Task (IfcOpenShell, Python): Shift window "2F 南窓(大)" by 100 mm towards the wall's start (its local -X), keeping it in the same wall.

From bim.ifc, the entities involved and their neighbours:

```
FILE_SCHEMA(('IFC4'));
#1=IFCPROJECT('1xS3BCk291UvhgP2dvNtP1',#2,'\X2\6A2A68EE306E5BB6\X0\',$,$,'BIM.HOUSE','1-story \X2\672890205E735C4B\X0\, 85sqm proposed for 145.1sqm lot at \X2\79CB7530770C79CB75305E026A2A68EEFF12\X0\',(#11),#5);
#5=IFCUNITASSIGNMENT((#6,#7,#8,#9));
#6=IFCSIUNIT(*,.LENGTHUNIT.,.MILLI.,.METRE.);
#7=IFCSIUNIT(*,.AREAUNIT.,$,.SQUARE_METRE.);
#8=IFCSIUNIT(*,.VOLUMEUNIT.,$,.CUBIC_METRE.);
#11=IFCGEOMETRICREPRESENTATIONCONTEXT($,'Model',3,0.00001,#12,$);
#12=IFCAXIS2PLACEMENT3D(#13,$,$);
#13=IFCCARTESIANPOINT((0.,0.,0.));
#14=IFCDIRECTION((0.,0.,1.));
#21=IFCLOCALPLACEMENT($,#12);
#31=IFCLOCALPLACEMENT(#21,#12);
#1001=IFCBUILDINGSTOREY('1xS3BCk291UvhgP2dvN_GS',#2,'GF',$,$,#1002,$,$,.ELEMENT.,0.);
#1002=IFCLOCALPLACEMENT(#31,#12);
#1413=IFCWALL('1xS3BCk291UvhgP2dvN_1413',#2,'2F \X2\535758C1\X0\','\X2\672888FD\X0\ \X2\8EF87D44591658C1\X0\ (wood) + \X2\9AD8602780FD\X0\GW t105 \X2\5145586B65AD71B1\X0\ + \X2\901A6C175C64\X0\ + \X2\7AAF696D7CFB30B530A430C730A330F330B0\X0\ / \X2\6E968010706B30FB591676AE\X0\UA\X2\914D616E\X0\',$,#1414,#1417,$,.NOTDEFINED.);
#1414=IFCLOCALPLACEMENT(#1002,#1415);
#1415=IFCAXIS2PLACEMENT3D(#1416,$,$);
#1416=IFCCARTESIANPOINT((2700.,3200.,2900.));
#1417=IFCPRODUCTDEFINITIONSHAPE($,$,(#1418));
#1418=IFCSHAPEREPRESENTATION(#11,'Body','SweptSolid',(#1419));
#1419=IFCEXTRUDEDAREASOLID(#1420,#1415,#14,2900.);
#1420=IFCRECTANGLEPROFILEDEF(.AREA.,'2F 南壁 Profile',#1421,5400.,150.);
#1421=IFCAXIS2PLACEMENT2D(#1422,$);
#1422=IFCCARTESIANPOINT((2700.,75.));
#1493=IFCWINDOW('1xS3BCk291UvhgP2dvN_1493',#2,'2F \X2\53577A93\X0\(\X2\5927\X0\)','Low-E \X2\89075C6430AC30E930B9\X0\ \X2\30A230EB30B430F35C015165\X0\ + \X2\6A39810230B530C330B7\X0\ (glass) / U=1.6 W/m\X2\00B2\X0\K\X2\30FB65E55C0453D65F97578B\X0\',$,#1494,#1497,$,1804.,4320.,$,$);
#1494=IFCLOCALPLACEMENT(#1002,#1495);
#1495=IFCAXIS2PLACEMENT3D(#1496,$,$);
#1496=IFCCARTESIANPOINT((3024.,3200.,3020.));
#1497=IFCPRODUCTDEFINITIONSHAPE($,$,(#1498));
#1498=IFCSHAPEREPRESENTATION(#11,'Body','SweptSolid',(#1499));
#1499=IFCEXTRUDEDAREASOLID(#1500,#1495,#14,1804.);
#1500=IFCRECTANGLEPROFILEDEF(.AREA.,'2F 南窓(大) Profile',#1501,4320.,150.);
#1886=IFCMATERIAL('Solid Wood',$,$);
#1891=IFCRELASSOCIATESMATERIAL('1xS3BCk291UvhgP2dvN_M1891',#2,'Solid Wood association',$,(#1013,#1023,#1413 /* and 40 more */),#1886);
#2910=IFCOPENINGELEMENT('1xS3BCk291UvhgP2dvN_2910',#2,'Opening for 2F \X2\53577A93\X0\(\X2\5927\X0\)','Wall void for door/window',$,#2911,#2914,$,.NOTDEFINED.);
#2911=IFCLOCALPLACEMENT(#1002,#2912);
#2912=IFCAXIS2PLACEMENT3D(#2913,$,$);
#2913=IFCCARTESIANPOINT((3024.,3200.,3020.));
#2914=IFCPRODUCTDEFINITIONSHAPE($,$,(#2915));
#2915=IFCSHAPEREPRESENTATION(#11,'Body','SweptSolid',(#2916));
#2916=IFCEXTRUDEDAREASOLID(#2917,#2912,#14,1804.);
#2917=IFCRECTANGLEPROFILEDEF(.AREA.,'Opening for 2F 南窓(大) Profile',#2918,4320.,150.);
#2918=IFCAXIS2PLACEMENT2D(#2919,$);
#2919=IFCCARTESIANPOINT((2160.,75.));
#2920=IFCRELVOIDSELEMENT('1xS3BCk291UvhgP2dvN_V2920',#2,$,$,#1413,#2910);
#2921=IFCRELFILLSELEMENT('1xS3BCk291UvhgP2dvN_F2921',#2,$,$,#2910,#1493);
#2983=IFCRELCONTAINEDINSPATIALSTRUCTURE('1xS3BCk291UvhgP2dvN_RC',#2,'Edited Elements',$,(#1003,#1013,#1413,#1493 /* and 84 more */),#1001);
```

```python
import ifcopenshell
import ifcopenshell.api.geometry
import ifcopenshell.util.placement
import ifcopenshell.util.unit

model = ifcopenshell.open("bim.ifc")
unit_scale = ifcopenshell.util.unit.calculate_unit_scale(model)

window = model.by_guid("1xS3BCk291UvhgP2dvN_1493")
opening = window.FillsVoids[0].RelatingOpeningElement
wall = opening.VoidsElements[0].RelatingBuildingElement

wall_matrix = ifcopenshell.util.placement.get_local_placement(wall.ObjectPlacement)
shift = wall_matrix[:3, 0] * -0.1 / unit_scale
before = ifcopenshell.util.placement.get_local_placement(window.ObjectPlacement)[:3, 3].copy()

# The window is not placed relative to its opening, so move both.
for product in (opening, window):
    matrix = ifcopenshell.util.placement.get_local_placement(product.ObjectPlacement)
    matrix[:3, 3] += shift
    ifcopenshell.api.geometry.edit_object_placement(model, product=product, matrix=matrix, is_si=False)

after = ifcopenshell.util.placement.get_local_placement(window.ObjectPlacement)[:3, 3]
print("window moved by", (after - before).round(3) + 0.0)

model.write("bim_updated.ifc")
```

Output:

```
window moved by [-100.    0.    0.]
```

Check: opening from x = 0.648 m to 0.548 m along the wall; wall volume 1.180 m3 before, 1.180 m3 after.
